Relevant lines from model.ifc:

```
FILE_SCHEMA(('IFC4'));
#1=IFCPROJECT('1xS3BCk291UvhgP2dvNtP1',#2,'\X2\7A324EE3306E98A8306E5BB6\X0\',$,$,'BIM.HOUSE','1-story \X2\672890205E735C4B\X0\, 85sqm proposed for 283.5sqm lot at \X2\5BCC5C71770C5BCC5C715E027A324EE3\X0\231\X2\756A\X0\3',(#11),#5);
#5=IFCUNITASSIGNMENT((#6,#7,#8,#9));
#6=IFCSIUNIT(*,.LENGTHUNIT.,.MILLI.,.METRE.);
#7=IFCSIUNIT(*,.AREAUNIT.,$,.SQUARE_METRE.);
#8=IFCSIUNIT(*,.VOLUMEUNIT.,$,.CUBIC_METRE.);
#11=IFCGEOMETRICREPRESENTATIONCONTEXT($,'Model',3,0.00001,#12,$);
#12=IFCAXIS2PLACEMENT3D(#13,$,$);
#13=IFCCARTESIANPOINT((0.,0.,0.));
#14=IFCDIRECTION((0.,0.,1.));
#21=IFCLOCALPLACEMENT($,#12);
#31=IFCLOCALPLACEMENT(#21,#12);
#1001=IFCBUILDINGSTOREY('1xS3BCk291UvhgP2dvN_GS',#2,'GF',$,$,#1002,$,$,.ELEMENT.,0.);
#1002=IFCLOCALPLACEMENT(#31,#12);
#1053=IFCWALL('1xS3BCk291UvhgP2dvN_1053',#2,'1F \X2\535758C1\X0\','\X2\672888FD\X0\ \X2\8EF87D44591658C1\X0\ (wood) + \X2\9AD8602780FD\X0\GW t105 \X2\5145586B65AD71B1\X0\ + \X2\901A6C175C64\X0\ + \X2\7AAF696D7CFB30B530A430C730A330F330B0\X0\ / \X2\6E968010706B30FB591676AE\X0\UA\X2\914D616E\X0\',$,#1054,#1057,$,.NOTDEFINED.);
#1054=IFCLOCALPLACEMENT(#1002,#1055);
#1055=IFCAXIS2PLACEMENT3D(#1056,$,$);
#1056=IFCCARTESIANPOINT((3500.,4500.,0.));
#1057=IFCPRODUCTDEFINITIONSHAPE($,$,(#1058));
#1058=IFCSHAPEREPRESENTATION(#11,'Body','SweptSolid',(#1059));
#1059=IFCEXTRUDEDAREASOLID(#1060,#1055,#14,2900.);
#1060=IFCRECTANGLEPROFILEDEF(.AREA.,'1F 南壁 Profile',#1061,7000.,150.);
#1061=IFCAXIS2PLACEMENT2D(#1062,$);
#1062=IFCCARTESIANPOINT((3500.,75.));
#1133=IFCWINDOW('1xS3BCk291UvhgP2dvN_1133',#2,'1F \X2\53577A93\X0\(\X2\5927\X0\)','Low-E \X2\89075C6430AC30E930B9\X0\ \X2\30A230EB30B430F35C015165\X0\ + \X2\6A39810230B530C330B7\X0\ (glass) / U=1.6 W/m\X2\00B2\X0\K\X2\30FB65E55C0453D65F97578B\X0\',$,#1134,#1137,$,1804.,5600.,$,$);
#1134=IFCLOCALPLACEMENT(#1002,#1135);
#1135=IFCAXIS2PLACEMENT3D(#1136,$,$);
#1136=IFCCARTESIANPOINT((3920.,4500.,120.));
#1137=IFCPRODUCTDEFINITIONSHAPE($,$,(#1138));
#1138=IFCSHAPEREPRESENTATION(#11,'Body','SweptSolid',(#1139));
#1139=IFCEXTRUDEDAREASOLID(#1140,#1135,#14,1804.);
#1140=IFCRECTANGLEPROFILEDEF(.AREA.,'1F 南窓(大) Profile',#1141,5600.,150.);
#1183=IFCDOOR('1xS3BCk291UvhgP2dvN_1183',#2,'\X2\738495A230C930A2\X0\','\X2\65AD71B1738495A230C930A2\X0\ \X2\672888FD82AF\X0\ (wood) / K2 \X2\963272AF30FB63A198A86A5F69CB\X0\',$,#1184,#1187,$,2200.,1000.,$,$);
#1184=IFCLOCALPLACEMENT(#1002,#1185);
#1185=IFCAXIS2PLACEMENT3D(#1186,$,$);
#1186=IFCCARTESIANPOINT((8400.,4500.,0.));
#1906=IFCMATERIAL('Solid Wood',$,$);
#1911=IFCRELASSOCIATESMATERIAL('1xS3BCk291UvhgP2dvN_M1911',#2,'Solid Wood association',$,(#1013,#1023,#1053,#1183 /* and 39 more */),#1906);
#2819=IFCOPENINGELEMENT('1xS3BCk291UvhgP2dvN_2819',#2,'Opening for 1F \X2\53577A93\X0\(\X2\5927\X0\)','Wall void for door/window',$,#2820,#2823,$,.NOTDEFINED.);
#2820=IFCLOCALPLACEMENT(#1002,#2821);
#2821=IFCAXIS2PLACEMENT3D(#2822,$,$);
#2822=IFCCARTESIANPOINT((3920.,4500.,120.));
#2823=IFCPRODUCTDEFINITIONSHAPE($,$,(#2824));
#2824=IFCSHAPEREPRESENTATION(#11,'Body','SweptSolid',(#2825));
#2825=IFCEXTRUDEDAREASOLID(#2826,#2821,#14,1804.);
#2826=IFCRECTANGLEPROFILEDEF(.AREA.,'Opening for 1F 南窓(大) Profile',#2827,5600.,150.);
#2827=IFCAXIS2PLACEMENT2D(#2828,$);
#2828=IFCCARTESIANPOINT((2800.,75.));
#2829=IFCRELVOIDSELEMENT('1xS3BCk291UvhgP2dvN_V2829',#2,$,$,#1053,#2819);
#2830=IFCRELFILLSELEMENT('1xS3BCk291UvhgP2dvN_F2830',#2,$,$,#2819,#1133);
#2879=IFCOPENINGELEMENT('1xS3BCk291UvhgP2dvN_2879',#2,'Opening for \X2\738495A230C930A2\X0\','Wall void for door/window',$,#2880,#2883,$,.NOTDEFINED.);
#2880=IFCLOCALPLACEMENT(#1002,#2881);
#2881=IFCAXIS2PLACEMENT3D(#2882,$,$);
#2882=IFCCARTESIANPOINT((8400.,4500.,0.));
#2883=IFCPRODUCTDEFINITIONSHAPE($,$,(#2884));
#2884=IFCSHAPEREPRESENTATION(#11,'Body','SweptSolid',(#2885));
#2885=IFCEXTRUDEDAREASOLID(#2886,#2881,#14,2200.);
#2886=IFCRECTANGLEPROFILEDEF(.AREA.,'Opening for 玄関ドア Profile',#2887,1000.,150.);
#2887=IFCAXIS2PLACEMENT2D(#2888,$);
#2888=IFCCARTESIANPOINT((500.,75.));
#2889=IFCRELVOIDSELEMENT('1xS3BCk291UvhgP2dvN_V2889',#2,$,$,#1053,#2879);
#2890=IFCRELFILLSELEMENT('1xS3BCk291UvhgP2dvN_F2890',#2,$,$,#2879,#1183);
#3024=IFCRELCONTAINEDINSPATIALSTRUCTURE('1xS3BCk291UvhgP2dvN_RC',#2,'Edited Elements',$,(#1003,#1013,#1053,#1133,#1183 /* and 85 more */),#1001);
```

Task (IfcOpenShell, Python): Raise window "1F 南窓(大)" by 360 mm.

```python
import numpy as np
import ifcopenshell
import ifcopenshell.api.geometry
import ifcopenshell.util.placement
import ifcopenshell.util.unit

model = ifcopenshell.open("model.ifc")
unit_scale = ifcopenshell.util.unit.calculate_unit_scale(model)

window = model.by_guid("1xS3BCk291UvhgP2dvN_1133")
opening = window.FillsVoids[0].RelatingOpeningElement
dz = 360.0

shift = np.array([0.0, 0.0, dz])
# The window is not placed relative to its opening, so move both.
for product in (opening, window):
    matrix = ifcopenshell.util.placement.get_local_placement(product.ObjectPlacement)
    matrix[:3, 3] += shift
    ifcopenshell.api.geometry.edit_object_placement(model, product=product, matrix=matrix, is_si=False)

print(f"moved by {dz * unit_scale:+.3f} m")

model.write("model-out.ifc")
```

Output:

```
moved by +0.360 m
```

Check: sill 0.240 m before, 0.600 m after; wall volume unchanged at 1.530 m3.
